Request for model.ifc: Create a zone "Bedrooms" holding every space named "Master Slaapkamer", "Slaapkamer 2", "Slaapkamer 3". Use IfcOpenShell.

First a look at what the model holds.

```python
import ifcopenshell

model = ifcopenshell.open("model.ifc")
print(model.schema)
seen = {}
for space in model.by_type("IfcSpace"):
    seen[space.LongName] = seen.get(space.LongName, 0) + 1
for name, count in sorted(seen.items(), key=str):
    print(count, "x", name)
print("zones:", [z.Name for z in model.by_type("IfcZone")][:20])
```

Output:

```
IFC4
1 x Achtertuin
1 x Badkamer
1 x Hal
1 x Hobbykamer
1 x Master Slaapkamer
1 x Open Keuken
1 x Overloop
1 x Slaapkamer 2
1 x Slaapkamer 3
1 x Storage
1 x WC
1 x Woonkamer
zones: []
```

```python
import ifcopenshell
import ifcopenshell.api.group
import ifcopenshell.api.root

model = ifcopenshell.open("model.ifc")

names = {"Master Slaapkamer", "Slaapkamer 2", "Slaapkamer 3"}
spaces = [s for s in model.by_type("IfcSpace") if s.LongName in names]

zone = ifcopenshell.api.root.create_entity(model, ifc_class="IfcZone", name="Bedrooms")
ifcopenshell.api.group.assign_group(model, products=spaces, group=zone)
print(len(spaces), "spaces in", zone.Name)

model.write("model_updated.ifc")
```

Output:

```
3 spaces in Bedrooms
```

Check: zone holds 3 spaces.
